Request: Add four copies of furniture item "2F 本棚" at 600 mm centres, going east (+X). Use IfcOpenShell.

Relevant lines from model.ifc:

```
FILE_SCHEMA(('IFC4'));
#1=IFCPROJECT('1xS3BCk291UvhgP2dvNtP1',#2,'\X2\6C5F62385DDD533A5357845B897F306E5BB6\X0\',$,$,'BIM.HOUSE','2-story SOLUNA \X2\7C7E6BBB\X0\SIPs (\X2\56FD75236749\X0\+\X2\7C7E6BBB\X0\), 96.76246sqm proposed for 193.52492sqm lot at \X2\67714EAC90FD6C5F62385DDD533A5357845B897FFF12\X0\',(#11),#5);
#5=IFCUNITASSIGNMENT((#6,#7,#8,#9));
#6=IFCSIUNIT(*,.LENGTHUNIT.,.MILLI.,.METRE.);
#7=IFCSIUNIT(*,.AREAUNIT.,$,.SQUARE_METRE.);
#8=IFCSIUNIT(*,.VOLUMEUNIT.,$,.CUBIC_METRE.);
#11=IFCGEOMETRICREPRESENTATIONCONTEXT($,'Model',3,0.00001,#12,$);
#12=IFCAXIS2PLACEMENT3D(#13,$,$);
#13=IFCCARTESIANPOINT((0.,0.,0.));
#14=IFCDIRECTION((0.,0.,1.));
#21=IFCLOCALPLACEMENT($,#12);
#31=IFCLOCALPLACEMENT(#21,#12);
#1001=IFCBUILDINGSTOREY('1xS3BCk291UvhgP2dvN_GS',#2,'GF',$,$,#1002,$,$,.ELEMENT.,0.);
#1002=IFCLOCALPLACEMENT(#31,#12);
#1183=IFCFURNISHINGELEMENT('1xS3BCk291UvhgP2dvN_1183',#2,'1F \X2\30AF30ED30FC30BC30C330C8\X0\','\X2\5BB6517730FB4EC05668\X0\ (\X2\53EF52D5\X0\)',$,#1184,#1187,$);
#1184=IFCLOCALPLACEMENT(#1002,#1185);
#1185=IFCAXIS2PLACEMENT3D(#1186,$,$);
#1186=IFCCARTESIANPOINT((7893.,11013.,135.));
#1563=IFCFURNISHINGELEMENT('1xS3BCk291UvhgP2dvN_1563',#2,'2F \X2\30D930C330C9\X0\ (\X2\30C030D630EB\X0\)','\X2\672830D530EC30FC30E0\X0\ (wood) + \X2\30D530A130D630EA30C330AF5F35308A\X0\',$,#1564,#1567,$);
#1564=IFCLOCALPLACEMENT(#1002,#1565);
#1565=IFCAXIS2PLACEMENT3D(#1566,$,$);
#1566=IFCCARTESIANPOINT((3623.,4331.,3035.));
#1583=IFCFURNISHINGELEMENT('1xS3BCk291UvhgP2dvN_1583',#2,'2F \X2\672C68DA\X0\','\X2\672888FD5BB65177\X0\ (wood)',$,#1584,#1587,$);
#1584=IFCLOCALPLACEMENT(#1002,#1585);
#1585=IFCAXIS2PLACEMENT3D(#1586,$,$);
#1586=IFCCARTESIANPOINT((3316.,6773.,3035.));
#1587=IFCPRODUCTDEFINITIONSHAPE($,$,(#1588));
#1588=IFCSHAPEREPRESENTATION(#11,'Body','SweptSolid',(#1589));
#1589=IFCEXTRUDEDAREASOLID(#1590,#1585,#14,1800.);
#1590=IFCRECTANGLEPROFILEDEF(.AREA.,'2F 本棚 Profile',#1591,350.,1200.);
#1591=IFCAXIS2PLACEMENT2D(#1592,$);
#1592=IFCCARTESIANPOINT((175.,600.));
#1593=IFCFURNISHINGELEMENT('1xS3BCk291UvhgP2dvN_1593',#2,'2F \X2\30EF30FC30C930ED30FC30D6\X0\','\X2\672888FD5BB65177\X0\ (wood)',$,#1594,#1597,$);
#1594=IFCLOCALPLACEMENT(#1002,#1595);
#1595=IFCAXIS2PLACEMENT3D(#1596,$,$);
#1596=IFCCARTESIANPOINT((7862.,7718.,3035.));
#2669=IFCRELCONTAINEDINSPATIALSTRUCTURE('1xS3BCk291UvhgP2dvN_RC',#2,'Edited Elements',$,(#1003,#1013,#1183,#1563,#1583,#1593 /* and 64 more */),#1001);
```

```python
import numpy as np
import ifcopenshell
import ifcopenshell.api.geometry
import ifcopenshell.api.root
import ifcopenshell.util.element
import ifcopenshell.util.placement
import ifcopenshell.util.unit

model = ifcopenshell.open("model.ifc")
unit_scale = ifcopenshell.util.unit.calculate_unit_scale(model)


def reuse_history(source, copy):
    """copy_class also copies each property set's owner history, people and application; keep the originals."""
    for rel in copy.IsDefinedBy:
        if rel.is_a("IfcRelDefinesByProperties") and (history := rel.RelatingPropertyDefinition.OwnerHistory):
            rel.RelatingPropertyDefinition.OwnerHistory = source.OwnerHistory
            ifcopenshell.util.element.remove_deep2(model, history)


source = model.by_guid("1xS3BCk291UvhgP2dvN_1583")
base = ifcopenshell.util.placement.get_local_placement(source.ObjectPlacement)
step = np.array([1.0, 0.0, 0.0]) * 0.6 / unit_scale

for i in range(1, 5):
    copy = ifcopenshell.api.root.copy_class(model, product=source)
    copy.Representation = ifcopenshell.util.element.copy_deep(
        model, source.Representation, exclude=["IfcGeometricRepresentationContext", "IfcRepresentationMap"]
    )
    reuse_history(source, copy)
    matrix = base.copy()
    matrix[:3, 3] += i * step
    print("added at", matrix[:3, 3].round(3) + 0.0)
    ifcopenshell.api.geometry.edit_object_placement(model, product=copy, matrix=matrix, is_si=False)

model.write("model_updated.ifc")
```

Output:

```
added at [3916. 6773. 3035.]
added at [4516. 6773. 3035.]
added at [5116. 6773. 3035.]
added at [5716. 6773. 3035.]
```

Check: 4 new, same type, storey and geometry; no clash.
